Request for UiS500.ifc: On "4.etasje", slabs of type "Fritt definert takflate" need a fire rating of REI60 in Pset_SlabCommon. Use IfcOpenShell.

First a look at what the model holds.

```python
import ifcopenshell
import ifcopenshell.util.element

model = ifcopenshell.open("UiS500.ifc")
print(model.schema)
storey = next(s for s in model.by_type("IfcBuildingStorey") if s.Name == "4.etasje")
slabs = [e for e in ifcopenshell.util.element.get_decomposition(storey) if e.is_a("IfcSlab")]
seen = {}
for e in slabs:
    element_type = ifcopenshell.util.element.get_type(e)
    key = (element_type.Name if element_type != e and element_type else None, ifcopenshell.util.element.get_pset(e, "Pset_SlabCommon", "FireRating"))
    seen[key] = seen.get(key, 0) + 1
for (name, value), count in sorted(seen.items(), key=str):
    print(count, "x", name, "|", value)
```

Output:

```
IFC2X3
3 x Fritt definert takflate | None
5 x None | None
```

```python
import ifcopenshell
import ifcopenshell.api.pset
import ifcopenshell.util.element

model = ifcopenshell.open("UiS500.ifc")

storey = next(s for s in model.by_type("IfcBuildingStorey") if s.Name == "4.etasje")
slabs = [e for e in ifcopenshell.util.element.get_decomposition(storey) if e.is_a("IfcSlab")]

count = 0
for e in slabs:
    element_type = ifcopenshell.util.element.get_type(e)
    if element_type in (None, e) or element_type.Name != "Fritt definert takflate":
        continue
    # add_pset returns the element's existing set when there is one.
    pset = ifcopenshell.api.pset.add_pset(model, product=e, name="Pset_SlabCommon")
    ifcopenshell.api.pset.edit_pset(model, pset=pset, properties={"FireRating": "REI60"})
    count += 1

print(count, "slabs updated")

model.write("UiS500_updated.ifc")
```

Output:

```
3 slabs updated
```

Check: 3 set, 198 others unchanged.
